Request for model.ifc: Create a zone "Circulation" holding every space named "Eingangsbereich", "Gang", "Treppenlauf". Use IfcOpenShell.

First a look at what the model holds.

```python
import ifcopenshell

model = ifcopenshell.open("model.ifc")
print(model.schema)
seen = {}
for space in model.by_type("IfcSpace"):
    seen[space.LongName] = seen.get(space.LongName, 0) + 1
for name, count in sorted(seen.items(), key=str):
    print(count, "x", name)
print("zones:", [z.Name for z in model.by_type("IfcZone")][:20])
```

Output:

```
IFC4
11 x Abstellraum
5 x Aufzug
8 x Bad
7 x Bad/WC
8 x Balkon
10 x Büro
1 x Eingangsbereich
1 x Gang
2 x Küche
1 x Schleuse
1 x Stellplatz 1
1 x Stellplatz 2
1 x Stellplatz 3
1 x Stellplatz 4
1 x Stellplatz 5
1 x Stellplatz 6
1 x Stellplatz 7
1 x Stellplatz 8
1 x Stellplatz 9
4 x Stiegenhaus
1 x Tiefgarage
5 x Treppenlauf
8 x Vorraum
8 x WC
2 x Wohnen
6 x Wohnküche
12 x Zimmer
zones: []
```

```python
import ifcopenshell
import ifcopenshell.api.group
import ifcopenshell.api.root

model = ifcopenshell.open("model.ifc")

names = {"Eingangsbereich", "Gang", "Treppenlauf"}
spaces = [s for s in model.by_type("IfcSpace") if s.LongName in names]

zone = ifcopenshell.api.root.create_entity(model, ifc_class="IfcZone", name="Circulation")
ifcopenshell.api.group.assign_group(model, products=spaces, group=zone)
print(len(spaces), "spaces in", zone.Name)

model.write("model-out.ifc")
```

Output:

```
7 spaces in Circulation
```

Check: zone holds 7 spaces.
